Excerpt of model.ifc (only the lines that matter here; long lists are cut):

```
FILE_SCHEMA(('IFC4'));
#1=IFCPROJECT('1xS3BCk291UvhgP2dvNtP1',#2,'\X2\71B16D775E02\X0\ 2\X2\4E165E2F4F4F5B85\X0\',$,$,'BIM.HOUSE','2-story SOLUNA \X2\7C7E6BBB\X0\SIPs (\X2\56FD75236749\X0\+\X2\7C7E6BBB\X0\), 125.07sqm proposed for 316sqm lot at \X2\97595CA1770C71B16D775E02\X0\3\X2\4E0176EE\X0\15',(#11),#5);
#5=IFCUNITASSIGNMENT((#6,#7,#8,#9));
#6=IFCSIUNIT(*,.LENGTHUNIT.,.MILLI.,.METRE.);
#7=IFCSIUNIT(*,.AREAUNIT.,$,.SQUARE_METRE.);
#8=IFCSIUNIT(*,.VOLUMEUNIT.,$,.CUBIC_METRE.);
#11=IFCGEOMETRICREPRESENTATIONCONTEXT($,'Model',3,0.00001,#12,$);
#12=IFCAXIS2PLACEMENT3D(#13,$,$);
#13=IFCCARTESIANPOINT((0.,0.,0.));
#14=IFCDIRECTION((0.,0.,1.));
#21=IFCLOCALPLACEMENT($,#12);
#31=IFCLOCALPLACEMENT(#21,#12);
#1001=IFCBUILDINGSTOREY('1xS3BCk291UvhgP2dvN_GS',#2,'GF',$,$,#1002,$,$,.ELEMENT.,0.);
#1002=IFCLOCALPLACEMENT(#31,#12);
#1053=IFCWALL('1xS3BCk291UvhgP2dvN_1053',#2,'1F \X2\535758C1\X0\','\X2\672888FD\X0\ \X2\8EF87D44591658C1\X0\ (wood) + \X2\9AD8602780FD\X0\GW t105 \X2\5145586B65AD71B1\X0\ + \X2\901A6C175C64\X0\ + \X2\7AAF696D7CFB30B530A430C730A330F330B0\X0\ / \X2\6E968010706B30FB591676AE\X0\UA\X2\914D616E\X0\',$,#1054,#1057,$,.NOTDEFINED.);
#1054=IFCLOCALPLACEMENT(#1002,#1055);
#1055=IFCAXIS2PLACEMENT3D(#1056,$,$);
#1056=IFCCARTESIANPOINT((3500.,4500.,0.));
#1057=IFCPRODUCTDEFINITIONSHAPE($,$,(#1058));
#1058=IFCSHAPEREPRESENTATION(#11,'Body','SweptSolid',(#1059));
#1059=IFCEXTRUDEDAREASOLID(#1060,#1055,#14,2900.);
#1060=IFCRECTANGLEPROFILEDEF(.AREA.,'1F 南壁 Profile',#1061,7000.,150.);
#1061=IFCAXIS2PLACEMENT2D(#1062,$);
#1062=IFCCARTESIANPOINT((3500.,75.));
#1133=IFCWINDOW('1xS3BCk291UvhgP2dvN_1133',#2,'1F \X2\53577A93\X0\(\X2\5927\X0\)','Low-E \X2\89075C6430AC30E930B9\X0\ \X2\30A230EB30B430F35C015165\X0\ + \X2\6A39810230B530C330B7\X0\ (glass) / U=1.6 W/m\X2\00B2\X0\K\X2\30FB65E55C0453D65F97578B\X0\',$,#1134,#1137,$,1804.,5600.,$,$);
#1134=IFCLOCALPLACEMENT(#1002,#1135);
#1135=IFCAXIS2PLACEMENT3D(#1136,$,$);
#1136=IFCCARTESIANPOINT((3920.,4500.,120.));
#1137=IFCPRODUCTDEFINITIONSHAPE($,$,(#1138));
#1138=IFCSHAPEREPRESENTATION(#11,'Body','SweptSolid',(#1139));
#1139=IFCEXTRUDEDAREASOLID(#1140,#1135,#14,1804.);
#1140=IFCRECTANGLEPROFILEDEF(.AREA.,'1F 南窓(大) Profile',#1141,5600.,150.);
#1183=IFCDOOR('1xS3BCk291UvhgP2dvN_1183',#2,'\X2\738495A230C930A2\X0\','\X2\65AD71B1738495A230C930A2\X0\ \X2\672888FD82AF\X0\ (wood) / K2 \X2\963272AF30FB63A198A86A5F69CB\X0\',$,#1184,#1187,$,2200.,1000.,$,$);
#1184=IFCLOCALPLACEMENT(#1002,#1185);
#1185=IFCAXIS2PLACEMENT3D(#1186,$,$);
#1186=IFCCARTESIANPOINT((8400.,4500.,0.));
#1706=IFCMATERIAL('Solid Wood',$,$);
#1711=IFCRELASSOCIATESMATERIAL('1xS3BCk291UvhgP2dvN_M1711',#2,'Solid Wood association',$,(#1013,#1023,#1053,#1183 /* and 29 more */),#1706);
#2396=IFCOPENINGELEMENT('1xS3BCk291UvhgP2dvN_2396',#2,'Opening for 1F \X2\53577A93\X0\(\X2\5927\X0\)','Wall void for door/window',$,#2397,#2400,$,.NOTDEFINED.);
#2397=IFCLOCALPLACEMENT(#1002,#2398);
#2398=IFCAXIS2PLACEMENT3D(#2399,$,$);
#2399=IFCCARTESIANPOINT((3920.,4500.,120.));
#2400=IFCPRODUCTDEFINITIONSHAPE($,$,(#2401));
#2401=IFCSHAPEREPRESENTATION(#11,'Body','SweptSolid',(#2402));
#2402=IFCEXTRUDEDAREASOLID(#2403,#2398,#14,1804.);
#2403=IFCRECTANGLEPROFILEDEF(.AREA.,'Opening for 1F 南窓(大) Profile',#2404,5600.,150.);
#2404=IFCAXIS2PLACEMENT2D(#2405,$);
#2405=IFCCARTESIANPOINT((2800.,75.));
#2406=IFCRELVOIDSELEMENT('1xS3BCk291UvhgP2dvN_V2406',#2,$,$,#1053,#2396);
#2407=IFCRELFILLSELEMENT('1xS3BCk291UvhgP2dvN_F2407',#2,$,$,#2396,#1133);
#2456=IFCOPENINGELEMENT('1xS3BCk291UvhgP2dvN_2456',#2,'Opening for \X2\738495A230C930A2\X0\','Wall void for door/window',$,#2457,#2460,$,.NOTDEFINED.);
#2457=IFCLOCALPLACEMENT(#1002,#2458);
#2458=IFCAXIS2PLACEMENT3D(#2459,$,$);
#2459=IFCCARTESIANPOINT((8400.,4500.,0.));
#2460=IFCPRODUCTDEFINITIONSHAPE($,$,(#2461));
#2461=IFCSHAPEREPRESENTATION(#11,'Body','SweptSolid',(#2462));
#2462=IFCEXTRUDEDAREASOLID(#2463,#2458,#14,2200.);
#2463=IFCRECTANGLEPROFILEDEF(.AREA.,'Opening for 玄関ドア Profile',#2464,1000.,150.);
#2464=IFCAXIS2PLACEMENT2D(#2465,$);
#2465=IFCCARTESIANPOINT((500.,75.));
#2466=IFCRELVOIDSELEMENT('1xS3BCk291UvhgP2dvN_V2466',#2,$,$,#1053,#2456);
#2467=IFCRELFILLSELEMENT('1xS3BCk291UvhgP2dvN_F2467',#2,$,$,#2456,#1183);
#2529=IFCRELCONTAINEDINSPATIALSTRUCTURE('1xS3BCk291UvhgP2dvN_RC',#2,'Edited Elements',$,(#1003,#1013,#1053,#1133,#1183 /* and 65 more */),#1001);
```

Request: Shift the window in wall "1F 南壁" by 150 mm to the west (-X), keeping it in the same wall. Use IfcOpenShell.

```python
import ifcopenshell
import ifcopenshell.api.geometry
import ifcopenshell.util.placement
import ifcopenshell.util.unit

model = ifcopenshell.open("model.ifc")
unit_scale = ifcopenshell.util.unit.calculate_unit_scale(model)

window = model.by_guid("1xS3BCk291UvhgP2dvN_1133")
opening = window.FillsVoids[0].RelatingOpeningElement
wall = opening.VoidsElements[0].RelatingBuildingElement

wall_matrix = ifcopenshell.util.placement.get_local_placement(wall.ObjectPlacement)
shift = wall_matrix[:3, 0] * -0.15 / unit_scale
before = ifcopenshell.util.placement.get_local_placement(window.ObjectPlacement)[:3, 3].copy()

# The window is not placed relative to its opening, so move both.
for product in (opening, window):
    matrix = ifcopenshell.util.placement.get_local_placement(product.ObjectPlacement)
    matrix[:3, 3] += shift
    ifcopenshell.api.geometry.edit_object_placement(model, product=product, matrix=matrix, is_si=False)

after = ifcopenshell.util.placement.get_local_placement(window.ObjectPlacement)[:3, 3]
print("window moved by", (after - before).round(3) + 0.0)

model.write("model_v2.ifc")
```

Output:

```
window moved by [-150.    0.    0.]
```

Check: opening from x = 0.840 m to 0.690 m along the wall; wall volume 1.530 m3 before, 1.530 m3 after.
